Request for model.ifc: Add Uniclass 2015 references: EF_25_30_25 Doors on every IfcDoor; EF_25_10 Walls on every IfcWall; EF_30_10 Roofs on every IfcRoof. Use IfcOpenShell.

First a look at what the model holds.

```python
import ifcopenshell

model = ifcopenshell.open("model.ifc")
print(model.schema)
print("classifications:", [c.Name for c in model.by_type("IfcClassification")])
for ifc_class in ("IfcDoor", "IfcRoof", "IfcStair", "IfcWall", "IfcWindow"):
    print(ifc_class, len(model.by_type(ifc_class)))
```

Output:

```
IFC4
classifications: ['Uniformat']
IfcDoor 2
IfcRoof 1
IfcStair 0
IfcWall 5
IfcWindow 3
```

```python
import ifcopenshell
import ifcopenshell.api.classification

model = ifcopenshell.open("model.ifc")

system = ifcopenshell.api.classification.add_classification(model, classification="Uniclass 2015")

codes = {
    "IfcDoor": ("EF_25_30_25", "Doors"),
    "IfcWall": ("EF_25_10", "Walls"),
    "IfcRoof": ("EF_30_10", "Roofs"),
}
for ifc_class, (code, name) in codes.items():
    products = model.by_type(ifc_class)
    ifcopenshell.api.classification.add_reference(
        model, products=products, classification=system, identification=code, name=name
    )
    print(code, len(products))

model.write("model_updated.ifc")
```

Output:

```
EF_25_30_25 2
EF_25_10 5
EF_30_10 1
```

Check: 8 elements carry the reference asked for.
